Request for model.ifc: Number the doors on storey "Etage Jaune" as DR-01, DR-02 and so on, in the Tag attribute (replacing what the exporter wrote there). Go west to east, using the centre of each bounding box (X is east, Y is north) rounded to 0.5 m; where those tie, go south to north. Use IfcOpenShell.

First a look at what the model holds.

```python
import ifcopenshell
import ifcopenshell.util.element
import ifcopenshell.util.placement

model = ifcopenshell.open("model.ifc")
print(model.schema)
storey = next(s for s in model.by_type("IfcBuildingStorey") if s.Name == "Etage Jaune")
doors = [e for e in ifcopenshell.util.element.get_decomposition(storey) if e.is_a("IfcDoor")]
for e in sorted(doors, key=lambda e: e.id()):
    origin = ifcopenshell.util.placement.get_local_placement(e.ObjectPlacement)[:3, 3]
    print(e.id(), e.Tag, e.Name, origin.round(2) + 0.0, sep=" | ")
```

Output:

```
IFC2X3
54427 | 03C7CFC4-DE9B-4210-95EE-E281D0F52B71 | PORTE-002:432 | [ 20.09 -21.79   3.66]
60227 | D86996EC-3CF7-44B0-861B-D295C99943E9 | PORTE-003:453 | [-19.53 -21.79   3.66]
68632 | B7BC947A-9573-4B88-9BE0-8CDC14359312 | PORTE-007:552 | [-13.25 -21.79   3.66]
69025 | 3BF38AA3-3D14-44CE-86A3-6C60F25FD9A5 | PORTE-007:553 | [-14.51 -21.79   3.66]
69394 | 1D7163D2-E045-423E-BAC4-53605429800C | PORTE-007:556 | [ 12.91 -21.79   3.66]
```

```python
import ifcopenshell
import ifcopenshell.geom
import ifcopenshell.util.element
import ifcopenshell.util.shape

model = ifcopenshell.open("model.ifc")
settings = ifcopenshell.geom.settings()
settings.set("use-world-coords", True)


def centre(element):
    shape = ifcopenshell.geom.create_shape(settings, element)
    return ifcopenshell.util.shape.get_bbox_centroid(shape.geometry)


storey = next(s for s in model.by_type("IfcBuildingStorey") if s.Name == "Etage Jaune")
doors = [e for e in ifcopenshell.util.element.get_decomposition(storey) if e.is_a("IfcDoor")]

# Insertion points can sit at a corner or the storey origin, so sort by the geometry (in metres).
centres = {e: centre(e) for e in doors}
doors.sort(key=lambda e: (round(centres[e][0] / 0.5), centres[e][1]))

for i, e in enumerate(doors, start=1):
    number = f"DR-{i:02d}"
    e.Tag = number
    print(e.id(), number)

model.write("model_v2.ifc")
```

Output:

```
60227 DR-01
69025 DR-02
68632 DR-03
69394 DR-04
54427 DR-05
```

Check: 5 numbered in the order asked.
